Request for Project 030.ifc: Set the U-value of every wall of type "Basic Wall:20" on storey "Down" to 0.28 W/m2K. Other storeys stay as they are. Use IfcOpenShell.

First a look at what the model holds.

```python
import ifcopenshell
import ifcopenshell.util.element

model = ifcopenshell.open("Project 030.ifc")
print(model.schema)
storey = next(s for s in model.by_type("IfcBuildingStorey") if s.Name == "Down")
walls = [e for e in ifcopenshell.util.element.get_decomposition(storey) if e.is_a("IfcWall")]
seen = {}
for e in walls:
    element_type = ifcopenshell.util.element.get_type(e)
    key = (element_type.Name if element_type != e and element_type else None, ifcopenshell.util.element.get_pset(e, "Pset_WallCommon", "ThermalTransmittance"))
    seen[key] = seen.get(key, 0) + 1
for (name, value), count in sorted(seen.items(), key=str):
    print(count, "x", name, "|", value)
```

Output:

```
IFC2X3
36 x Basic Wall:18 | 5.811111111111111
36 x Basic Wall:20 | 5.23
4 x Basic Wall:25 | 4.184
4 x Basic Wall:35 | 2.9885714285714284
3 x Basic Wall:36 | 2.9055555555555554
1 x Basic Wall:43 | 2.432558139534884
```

```python
import ifcopenshell
import ifcopenshell.api.pset
import ifcopenshell.util.element

model = ifcopenshell.open("Project 030.ifc")

storey = next(s for s in model.by_type("IfcBuildingStorey") if s.Name == "Down")
walls = [e for e in ifcopenshell.util.element.get_decomposition(storey) if e.is_a("IfcWall")]

count = 0
for e in walls:
    element_type = ifcopenshell.util.element.get_type(e)
    if element_type in (None, e) or element_type.Name != "Basic Wall:20":
        continue
    # add_pset returns the element's existing set when there is one.
    pset = ifcopenshell.api.pset.add_pset(model, product=e, name="Pset_WallCommon")
    ifcopenshell.api.pset.edit_pset(model, pset=pset, properties={"ThermalTransmittance": 0.28})
    count += 1

print(count, "walls updated")

model.write("Project 030_v2.ifc")
```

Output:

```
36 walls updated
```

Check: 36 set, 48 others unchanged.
